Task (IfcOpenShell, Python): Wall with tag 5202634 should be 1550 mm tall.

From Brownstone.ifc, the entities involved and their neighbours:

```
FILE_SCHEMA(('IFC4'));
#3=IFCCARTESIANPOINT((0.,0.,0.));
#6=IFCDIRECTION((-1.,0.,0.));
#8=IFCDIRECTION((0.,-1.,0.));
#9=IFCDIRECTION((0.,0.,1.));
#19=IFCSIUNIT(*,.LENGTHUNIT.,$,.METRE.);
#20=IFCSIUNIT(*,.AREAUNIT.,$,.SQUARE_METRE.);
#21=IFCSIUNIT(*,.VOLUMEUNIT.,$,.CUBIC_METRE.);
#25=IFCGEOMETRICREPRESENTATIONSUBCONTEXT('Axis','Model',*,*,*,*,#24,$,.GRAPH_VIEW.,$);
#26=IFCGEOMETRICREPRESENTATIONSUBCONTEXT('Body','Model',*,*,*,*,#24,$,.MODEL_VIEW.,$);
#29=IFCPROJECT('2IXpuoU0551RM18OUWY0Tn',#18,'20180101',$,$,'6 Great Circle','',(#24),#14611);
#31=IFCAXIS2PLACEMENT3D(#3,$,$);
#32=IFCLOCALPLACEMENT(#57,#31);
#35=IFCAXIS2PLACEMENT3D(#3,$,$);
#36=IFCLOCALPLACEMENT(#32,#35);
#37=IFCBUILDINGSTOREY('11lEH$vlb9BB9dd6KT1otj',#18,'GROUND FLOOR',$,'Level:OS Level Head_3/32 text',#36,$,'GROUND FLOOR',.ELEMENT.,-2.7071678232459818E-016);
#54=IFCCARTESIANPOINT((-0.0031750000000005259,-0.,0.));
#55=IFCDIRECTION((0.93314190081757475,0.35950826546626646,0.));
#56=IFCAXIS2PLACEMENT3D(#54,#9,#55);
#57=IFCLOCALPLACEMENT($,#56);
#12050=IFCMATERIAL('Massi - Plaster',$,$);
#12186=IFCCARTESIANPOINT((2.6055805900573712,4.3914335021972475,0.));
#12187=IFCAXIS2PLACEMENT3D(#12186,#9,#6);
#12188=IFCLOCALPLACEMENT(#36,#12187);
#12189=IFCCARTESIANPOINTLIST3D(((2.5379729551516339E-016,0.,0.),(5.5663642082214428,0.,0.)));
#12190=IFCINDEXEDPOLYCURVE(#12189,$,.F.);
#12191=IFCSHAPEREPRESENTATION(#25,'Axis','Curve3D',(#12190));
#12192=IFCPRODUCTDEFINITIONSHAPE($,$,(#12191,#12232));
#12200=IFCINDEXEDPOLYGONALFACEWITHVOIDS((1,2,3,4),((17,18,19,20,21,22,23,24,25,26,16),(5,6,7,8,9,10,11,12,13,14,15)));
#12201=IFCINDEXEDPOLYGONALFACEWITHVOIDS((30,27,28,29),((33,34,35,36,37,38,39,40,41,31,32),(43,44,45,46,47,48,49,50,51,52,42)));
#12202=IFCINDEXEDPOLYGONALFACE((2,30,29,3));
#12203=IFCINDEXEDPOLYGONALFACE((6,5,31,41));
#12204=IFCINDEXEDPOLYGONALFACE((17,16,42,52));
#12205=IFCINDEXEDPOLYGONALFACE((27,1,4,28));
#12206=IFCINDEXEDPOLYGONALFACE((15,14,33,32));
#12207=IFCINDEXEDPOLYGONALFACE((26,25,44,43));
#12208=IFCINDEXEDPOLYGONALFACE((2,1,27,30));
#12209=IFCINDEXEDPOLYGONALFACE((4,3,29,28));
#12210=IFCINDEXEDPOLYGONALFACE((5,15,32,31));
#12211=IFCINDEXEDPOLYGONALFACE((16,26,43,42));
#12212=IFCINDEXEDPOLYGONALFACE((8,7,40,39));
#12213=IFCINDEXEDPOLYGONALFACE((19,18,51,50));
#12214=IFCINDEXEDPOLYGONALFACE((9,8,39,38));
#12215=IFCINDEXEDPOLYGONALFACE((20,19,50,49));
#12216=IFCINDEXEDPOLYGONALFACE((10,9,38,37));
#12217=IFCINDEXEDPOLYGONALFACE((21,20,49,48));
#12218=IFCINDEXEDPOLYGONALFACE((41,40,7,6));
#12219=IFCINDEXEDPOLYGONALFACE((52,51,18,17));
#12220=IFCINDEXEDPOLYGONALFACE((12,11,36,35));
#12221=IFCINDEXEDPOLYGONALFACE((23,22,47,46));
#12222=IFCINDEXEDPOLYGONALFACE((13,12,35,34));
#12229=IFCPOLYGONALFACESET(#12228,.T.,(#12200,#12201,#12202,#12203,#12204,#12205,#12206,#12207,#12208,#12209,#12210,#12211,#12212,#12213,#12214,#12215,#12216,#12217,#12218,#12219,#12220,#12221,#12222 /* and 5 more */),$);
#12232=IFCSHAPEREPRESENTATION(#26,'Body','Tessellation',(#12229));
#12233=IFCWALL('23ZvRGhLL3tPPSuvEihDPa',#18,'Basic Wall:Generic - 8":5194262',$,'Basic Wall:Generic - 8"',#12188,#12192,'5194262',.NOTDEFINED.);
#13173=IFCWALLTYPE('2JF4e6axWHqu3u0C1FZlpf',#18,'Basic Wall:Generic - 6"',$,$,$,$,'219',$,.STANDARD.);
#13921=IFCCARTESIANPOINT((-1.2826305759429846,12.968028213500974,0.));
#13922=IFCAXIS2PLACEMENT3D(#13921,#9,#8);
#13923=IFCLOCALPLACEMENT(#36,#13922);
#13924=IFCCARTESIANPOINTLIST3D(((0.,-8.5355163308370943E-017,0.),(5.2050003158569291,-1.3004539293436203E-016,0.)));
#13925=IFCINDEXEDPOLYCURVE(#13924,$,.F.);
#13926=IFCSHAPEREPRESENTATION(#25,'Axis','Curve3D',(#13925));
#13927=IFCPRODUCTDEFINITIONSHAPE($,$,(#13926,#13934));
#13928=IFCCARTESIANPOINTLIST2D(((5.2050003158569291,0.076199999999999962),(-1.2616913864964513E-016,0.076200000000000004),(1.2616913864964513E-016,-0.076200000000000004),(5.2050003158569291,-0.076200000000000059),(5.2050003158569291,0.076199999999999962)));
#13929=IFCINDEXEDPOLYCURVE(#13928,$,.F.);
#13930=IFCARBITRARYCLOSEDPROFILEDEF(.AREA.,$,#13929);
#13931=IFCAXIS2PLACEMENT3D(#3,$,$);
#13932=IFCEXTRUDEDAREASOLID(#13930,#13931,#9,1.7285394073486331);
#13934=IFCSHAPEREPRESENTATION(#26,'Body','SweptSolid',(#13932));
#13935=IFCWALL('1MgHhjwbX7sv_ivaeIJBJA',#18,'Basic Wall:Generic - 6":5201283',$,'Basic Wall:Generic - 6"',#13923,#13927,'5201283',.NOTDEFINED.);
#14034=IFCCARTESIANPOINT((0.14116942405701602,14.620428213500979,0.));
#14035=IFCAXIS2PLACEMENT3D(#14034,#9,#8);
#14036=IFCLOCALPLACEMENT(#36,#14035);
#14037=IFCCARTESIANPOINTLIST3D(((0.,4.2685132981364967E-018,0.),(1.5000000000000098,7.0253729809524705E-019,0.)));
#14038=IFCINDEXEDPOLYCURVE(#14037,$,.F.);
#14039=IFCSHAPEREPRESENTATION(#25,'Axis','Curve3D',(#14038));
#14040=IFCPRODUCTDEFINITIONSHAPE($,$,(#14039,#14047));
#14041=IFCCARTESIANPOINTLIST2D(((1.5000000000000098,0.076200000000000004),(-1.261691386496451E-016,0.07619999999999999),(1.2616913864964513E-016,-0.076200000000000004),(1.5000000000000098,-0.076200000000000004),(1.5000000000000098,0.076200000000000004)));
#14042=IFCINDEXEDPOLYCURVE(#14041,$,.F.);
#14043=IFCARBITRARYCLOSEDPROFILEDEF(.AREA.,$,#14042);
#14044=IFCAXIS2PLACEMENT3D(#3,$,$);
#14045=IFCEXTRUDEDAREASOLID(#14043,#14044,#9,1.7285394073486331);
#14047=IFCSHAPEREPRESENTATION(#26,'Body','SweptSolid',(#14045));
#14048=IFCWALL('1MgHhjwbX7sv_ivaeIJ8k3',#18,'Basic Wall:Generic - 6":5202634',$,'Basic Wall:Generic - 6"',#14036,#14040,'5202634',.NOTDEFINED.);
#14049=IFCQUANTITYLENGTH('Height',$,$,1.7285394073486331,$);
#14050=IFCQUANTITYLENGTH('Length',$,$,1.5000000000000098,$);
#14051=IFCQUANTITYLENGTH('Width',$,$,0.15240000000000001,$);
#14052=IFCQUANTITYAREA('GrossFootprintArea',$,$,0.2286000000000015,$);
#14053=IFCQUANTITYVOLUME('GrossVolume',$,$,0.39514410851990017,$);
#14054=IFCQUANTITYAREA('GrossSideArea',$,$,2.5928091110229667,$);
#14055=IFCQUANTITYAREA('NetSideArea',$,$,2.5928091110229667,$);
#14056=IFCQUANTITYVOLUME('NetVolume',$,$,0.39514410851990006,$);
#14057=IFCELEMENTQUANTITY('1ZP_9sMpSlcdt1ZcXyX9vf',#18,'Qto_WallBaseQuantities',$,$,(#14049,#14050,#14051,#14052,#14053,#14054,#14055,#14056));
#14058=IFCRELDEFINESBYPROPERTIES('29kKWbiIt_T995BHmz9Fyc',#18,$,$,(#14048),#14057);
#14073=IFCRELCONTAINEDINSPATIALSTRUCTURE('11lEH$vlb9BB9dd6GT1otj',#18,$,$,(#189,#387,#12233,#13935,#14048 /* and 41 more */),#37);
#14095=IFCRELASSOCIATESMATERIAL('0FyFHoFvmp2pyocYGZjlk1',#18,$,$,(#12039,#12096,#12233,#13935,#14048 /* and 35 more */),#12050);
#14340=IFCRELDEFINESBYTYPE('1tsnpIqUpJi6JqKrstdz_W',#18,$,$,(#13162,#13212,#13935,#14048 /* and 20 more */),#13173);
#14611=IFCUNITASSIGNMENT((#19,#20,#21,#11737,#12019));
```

```python
import ifcopenshell
import ifcopenshell.api.pset
import ifcopenshell.geom
import ifcopenshell.util.element
import ifcopenshell.util.representation
import ifcopenshell.util.shape
import ifcopenshell.util.unit

model = ifcopenshell.open("Brownstone.ifc")
unit_scale = ifcopenshell.util.unit.calculate_unit_scale(model)
area_scale = ifcopenshell.util.unit.calculate_unit_scale(model, "AREAUNIT")
volume_scale = ifcopenshell.util.unit.calculate_unit_scale(model, "VOLUMEUNIT")
settings = ifcopenshell.geom.settings()


def volume(element):
    """Net volume in cubic metres, openings subtracted."""
    shape = ifcopenshell.geom.create_shape(settings, element)
    return ifcopenshell.util.shape.get_volume(shape.geometry)


wall = model.by_id(14048)
before = volume(wall)

body = ifcopenshell.util.representation.get_representation(wall, "Model", "Body")
solid = body.Items[0]
old_height = solid.Depth
solid.Depth = 1.55 / unit_scale
after = volume(wall)
thickness = 0.1524  # wall thickness in metres

# Update the stored height, areas and volumes.
qto = model.by_id(ifcopenshell.util.element.get_pset(wall, "Qto_WallBaseQuantities", should_inherit=False)["id"])
ifcopenshell.api.pset.edit_qto(model, qto=qto, properties={
    "Height": solid.Depth,
    "GrossVolume": ifcopenshell.util.element.get_pset(wall, "Qto_WallBaseQuantities", "GrossVolume") * solid.Depth / old_height,
    "GrossSideArea": ifcopenshell.util.element.get_pset(wall, "Qto_WallBaseQuantities", "GrossSideArea") * solid.Depth / old_height,
    "NetSideArea": after / thickness / area_scale,
    "NetVolume": after / volume_scale,
})

print(f"height {old_height:g} -> {solid.Depth:g}, volume {before:.3f} -> {after:.3f} m3")

model.write("Brownstone_v2.ifc")
```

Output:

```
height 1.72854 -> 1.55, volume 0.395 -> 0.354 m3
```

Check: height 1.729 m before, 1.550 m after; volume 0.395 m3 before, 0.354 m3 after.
